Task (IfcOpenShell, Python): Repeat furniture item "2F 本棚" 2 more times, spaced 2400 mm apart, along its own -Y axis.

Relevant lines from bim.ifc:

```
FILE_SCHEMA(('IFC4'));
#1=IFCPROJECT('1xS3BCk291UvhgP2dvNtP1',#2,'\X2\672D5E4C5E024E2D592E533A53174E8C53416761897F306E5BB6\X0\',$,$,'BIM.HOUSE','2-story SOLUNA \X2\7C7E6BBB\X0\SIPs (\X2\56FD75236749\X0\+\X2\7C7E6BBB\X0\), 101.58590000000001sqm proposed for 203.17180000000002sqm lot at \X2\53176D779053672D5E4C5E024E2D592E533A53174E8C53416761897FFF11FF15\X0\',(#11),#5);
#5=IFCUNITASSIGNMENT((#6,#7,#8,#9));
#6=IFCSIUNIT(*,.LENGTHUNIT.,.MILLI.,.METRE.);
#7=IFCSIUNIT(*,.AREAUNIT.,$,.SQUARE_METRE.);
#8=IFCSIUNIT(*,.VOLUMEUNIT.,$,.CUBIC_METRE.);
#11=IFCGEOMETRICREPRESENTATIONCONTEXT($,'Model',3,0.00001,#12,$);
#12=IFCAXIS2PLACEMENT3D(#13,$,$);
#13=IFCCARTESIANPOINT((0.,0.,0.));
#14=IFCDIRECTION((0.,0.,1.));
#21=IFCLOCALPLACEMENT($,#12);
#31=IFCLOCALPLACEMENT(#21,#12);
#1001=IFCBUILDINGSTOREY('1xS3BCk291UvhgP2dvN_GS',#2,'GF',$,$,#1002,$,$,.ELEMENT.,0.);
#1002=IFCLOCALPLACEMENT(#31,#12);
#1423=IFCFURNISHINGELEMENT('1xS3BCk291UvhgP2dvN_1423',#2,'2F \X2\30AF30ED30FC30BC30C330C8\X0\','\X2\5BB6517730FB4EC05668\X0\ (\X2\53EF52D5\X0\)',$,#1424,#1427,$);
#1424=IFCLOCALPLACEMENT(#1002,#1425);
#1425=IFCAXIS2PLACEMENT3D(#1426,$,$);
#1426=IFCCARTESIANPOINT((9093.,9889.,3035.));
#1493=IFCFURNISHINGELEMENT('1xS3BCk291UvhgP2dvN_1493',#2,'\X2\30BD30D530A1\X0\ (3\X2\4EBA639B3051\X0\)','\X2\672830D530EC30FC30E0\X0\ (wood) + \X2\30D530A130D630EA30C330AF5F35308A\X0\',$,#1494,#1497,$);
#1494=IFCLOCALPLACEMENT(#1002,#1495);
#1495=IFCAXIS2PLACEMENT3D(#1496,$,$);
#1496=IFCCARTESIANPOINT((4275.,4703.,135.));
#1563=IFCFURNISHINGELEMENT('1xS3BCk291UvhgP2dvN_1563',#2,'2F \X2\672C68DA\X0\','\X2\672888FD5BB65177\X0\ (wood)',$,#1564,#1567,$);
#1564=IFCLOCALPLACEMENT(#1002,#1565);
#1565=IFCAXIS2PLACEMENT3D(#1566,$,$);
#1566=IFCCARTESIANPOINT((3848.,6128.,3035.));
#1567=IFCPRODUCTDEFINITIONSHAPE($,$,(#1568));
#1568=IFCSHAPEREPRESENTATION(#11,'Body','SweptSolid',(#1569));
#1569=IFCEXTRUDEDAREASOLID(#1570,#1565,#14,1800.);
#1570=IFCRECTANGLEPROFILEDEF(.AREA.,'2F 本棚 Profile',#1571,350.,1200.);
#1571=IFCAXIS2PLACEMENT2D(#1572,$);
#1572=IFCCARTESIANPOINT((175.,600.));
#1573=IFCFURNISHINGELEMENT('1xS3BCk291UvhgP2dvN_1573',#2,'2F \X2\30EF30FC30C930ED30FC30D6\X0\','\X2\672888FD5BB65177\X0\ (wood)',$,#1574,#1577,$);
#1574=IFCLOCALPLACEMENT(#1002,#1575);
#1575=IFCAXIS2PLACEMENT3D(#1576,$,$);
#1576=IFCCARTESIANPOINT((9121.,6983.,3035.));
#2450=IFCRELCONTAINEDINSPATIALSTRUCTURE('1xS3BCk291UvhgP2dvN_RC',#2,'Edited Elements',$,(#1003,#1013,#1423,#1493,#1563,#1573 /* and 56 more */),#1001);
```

```python
import ifcopenshell
import ifcopenshell.api.geometry
import ifcopenshell.api.root
import ifcopenshell.util.element
import ifcopenshell.util.placement
import ifcopenshell.util.unit

model = ifcopenshell.open("bim.ifc")
unit_scale = ifcopenshell.util.unit.calculate_unit_scale(model)


def reuse_history(source, copy):
    """copy_class also copies each property set's owner history, people and application; keep the originals."""
    for rel in copy.IsDefinedBy:
        if rel.is_a("IfcRelDefinesByProperties") and (history := rel.RelatingPropertyDefinition.OwnerHistory):
            rel.RelatingPropertyDefinition.OwnerHistory = source.OwnerHistory
            ifcopenshell.util.element.remove_deep2(model, history)


source = model.by_guid("1xS3BCk291UvhgP2dvN_1563")
base = ifcopenshell.util.placement.get_local_placement(source.ObjectPlacement)
step = -base[:3, 1] * 2.4 / unit_scale

for i in range(1, 3):
    copy = ifcopenshell.api.root.copy_class(model, product=source)
    copy.Representation = ifcopenshell.util.element.copy_deep(
        model, source.Representation, exclude=["IfcGeometricRepresentationContext", "IfcRepresentationMap"]
    )
    reuse_history(source, copy)
    matrix = base.copy()
    matrix[:3, 3] += i * step
    print("added at", matrix[:3, 3].round(3) + 0.0)
    ifcopenshell.api.geometry.edit_object_placement(model, product=copy, matrix=matrix, is_si=False)

model.write("bim_edited.ifc")
```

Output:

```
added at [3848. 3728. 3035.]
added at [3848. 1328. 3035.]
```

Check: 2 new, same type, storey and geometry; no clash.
